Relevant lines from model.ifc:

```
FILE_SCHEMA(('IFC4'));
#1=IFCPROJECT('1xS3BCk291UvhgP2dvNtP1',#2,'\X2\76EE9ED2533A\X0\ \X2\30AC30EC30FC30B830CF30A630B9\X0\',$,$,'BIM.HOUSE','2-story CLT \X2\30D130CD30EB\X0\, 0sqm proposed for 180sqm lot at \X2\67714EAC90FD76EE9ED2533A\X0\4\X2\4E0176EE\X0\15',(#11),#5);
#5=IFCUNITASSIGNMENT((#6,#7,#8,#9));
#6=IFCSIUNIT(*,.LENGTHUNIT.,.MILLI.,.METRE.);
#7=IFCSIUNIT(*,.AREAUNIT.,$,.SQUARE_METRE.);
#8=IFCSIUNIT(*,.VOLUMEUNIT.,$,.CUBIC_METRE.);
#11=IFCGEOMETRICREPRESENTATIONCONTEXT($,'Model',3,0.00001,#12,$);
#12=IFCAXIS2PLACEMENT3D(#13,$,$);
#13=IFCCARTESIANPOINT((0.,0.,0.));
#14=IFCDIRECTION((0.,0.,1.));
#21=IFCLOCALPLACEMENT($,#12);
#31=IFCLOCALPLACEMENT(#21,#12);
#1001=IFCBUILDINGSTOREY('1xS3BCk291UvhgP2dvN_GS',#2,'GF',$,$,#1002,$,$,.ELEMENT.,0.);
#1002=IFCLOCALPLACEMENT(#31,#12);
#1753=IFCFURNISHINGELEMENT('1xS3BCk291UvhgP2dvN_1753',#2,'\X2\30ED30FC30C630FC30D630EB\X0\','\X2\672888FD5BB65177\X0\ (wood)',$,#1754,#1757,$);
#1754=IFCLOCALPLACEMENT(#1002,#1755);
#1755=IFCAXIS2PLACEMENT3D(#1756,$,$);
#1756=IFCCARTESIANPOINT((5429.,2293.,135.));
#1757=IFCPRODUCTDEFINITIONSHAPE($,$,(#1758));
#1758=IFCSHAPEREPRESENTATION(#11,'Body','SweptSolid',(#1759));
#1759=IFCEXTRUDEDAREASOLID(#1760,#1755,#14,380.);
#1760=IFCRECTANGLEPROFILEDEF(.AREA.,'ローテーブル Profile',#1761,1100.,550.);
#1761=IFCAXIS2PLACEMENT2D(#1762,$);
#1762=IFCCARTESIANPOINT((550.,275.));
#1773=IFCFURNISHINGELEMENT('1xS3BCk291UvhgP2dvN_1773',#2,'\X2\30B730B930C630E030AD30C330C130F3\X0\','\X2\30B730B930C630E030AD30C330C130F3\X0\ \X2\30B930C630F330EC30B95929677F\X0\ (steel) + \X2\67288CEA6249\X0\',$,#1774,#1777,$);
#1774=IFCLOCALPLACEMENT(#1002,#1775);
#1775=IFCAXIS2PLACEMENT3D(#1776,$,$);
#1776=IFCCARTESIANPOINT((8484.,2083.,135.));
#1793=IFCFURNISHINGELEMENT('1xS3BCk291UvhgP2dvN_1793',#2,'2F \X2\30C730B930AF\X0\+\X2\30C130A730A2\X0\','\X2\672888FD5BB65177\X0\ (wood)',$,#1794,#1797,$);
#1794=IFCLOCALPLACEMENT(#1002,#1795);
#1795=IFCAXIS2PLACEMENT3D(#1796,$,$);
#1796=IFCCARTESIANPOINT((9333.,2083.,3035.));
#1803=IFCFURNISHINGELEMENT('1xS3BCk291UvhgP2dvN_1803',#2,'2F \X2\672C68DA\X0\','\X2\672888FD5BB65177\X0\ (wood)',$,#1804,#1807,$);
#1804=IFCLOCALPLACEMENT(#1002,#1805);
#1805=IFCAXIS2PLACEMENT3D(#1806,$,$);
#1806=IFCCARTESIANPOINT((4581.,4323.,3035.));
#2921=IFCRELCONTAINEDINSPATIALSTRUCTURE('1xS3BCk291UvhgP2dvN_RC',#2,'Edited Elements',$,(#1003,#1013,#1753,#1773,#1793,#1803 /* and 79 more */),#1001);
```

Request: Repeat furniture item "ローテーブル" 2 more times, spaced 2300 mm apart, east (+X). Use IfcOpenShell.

```python
import numpy as np
import ifcopenshell
import ifcopenshell.api.geometry
import ifcopenshell.api.root
import ifcopenshell.util.element
import ifcopenshell.util.placement
import ifcopenshell.util.unit

model = ifcopenshell.open("model.ifc")
unit_scale = ifcopenshell.util.unit.calculate_unit_scale(model)


def reuse_history(source, copy):
    """copy_class also copies each property set's owner history, people and application; keep the originals."""
    for rel in copy.IsDefinedBy:
        if rel.is_a("IfcRelDefinesByProperties") and (history := rel.RelatingPropertyDefinition.OwnerHistory):
            rel.RelatingPropertyDefinition.OwnerHistory = source.OwnerHistory
            ifcopenshell.util.element.remove_deep2(model, history)


source = model.by_guid("1xS3BCk291UvhgP2dvN_1753")
base = ifcopenshell.util.placement.get_local_placement(source.ObjectPlacement)
step = np.array([1.0, 0.0, 0.0]) * 2.3 / unit_scale

for i in range(1, 3):
    copy = ifcopenshell.api.root.copy_class(model, product=source)
    copy.Representation = ifcopenshell.util.element.copy_deep(
        model, source.Representation, exclude=["IfcGeometricRepresentationContext", "IfcRepresentationMap"]
    )
    reuse_history(source, copy)
    matrix = base.copy()
    matrix[:3, 3] += i * step
    print("added at", matrix[:3, 3].round(3) + 0.0)
    ifcopenshell.api.geometry.edit_object_placement(model, product=copy, matrix=matrix, is_si=False)

model.write("model_v2.ifc")
```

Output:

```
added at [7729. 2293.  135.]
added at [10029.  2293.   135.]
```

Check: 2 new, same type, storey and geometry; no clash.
